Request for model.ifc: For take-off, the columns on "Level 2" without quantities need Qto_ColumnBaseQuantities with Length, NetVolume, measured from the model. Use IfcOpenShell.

First a look at what the model holds.

```python
import ifcopenshell
import ifcopenshell.util.element
import ifcopenshell.util.unit

model = ifcopenshell.open("model.ifc")
print(model.schema)
for unit_type in ("LENGTHUNIT", "AREAUNIT", "VOLUMEUNIT"):
    print(unit_type, ifcopenshell.util.unit.calculate_unit_scale(model, unit_type))
storey = next(s for s in model.by_type("IfcBuildingStorey") if s.Name == "Level 2")
columns = [e for e in ifcopenshell.util.element.get_decomposition(storey) if e.is_a("IfcColumn")]
for e in sorted(columns, key=lambda e: e.id()):
    print(e.id(), e.is_a(), e.Name, list(ifcopenshell.util.element.get_psets(e, qtos_only=True)), sep=" | ")
```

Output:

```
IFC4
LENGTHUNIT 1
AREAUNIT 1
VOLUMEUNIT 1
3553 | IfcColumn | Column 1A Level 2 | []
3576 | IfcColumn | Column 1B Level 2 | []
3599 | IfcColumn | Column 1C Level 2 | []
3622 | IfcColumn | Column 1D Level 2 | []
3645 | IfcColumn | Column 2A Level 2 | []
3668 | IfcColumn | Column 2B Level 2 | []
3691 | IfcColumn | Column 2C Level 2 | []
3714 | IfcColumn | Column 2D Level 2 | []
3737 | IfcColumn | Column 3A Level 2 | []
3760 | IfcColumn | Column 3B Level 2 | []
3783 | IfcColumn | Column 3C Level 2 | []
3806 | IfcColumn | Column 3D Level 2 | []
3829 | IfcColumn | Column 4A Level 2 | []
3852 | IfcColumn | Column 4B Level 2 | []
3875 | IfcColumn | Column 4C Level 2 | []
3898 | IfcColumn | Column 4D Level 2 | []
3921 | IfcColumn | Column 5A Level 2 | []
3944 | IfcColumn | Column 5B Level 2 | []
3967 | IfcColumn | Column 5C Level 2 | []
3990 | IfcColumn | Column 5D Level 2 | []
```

```python
import ifcopenshell
import ifcopenshell.api.pset
import ifcopenshell.geom
import ifcopenshell.util.element
import ifcopenshell.util.shape
import ifcopenshell.util.unit

model = ifcopenshell.open("model.ifc")
unit_scale = ifcopenshell.util.unit.calculate_unit_scale(model)
volume_scale = ifcopenshell.util.unit.calculate_unit_scale(model, "VOLUMEUNIT")
settings = ifcopenshell.geom.settings()

storey = next(s for s in model.by_type("IfcBuildingStorey") if s.Name == "Level 2")
columns = [e for e in ifcopenshell.util.element.get_decomposition(storey) if e.is_a("IfcColumn")]

for e in sorted(columns, key=lambda e: e.id()):
    if ifcopenshell.util.element.get_psets(e, qtos_only=True, should_inherit=False):
        continue
    # Geometry comes back in metres, in the element's own axes.
    shape = ifcopenshell.geom.create_shape(settings, e)
    values = {
        "Length": ifcopenshell.util.shape.get_z(shape.geometry) / unit_scale,
        "NetVolume": ifcopenshell.util.shape.get_volume(shape.geometry) / volume_scale,
    }
    qto = ifcopenshell.api.pset.add_qto(model, product=e, name="Qto_ColumnBaseQuantities")
    ifcopenshell.api.pset.edit_qto(model, qto=qto, properties=values)
    print(e.id(), {k: round(v, 3) for k, v in values.items()})

model.write("model_updated.ifc")
```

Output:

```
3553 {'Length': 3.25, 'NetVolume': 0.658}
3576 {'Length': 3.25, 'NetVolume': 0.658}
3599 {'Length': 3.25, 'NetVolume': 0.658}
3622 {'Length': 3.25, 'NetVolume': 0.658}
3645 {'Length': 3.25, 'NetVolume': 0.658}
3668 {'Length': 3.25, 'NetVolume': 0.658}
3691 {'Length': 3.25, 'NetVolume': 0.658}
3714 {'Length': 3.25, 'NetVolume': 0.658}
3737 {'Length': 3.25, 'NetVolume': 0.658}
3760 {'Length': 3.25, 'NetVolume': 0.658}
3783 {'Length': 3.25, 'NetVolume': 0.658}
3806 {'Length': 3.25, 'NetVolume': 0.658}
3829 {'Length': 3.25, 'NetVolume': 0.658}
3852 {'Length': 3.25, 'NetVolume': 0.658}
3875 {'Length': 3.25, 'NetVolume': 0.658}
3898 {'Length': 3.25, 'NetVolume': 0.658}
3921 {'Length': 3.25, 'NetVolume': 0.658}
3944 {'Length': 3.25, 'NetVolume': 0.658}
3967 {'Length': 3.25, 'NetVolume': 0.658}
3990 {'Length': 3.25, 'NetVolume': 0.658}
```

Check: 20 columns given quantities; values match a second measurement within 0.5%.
